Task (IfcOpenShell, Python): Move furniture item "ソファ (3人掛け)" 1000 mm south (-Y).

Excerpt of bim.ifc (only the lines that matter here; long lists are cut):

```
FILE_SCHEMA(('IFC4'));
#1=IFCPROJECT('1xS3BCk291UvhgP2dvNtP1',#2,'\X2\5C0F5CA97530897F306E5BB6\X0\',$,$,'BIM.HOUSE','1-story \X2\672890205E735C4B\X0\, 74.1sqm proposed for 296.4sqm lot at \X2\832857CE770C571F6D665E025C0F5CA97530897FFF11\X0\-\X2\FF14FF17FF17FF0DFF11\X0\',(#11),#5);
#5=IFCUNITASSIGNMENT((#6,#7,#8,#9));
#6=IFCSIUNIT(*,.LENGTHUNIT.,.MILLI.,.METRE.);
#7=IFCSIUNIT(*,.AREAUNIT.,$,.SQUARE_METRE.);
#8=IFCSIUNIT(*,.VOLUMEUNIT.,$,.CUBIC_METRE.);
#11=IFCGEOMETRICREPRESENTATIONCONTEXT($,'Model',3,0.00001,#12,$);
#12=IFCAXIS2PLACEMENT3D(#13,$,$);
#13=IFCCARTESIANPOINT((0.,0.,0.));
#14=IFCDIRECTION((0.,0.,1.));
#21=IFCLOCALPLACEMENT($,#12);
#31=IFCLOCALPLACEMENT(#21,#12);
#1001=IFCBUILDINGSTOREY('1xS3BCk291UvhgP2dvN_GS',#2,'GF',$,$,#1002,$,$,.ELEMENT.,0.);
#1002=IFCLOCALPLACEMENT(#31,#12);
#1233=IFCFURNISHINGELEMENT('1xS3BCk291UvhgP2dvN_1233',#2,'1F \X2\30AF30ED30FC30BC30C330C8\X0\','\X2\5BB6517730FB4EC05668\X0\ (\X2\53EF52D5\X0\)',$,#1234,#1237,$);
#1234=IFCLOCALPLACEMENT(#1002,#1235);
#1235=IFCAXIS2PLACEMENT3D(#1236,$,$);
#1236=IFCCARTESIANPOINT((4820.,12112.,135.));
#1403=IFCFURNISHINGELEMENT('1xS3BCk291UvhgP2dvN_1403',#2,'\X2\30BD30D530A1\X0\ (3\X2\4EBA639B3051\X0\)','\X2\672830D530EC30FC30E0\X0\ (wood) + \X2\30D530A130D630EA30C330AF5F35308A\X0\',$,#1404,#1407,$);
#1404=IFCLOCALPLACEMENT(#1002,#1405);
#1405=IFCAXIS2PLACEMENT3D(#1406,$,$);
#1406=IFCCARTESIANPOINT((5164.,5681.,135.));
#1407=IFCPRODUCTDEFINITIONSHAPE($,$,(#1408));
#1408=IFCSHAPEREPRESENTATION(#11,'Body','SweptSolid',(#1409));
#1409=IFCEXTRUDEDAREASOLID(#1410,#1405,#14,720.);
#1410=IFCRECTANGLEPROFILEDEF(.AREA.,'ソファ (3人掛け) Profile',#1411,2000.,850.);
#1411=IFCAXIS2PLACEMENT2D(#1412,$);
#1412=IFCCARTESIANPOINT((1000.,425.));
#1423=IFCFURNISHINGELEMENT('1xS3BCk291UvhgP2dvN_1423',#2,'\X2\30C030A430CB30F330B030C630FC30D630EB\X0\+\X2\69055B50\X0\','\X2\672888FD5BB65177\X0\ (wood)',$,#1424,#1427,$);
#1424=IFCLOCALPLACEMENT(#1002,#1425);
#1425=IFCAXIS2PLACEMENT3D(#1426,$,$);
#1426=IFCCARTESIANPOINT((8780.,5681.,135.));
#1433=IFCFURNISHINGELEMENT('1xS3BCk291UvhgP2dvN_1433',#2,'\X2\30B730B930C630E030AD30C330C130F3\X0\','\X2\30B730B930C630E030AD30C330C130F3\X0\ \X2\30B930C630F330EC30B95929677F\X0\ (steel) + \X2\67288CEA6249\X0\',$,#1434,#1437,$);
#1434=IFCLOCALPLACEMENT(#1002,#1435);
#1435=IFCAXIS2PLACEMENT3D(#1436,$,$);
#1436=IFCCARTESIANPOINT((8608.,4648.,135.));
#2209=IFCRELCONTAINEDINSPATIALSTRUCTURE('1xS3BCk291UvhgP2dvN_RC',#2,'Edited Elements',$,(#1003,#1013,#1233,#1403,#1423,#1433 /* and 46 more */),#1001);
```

```python
import ifcopenshell
import ifcopenshell.api.geometry
import ifcopenshell.util.placement
import ifcopenshell.util.unit

model = ifcopenshell.open("bim.ifc")
unit_scale = ifcopenshell.util.unit.calculate_unit_scale(model)

item = model.by_id(1403)
matrix = ifcopenshell.util.placement.get_local_placement(item.ObjectPlacement)
matrix[1, 3] -= 1 / unit_scale
ifcopenshell.api.geometry.edit_object_placement(model, product=item, matrix=matrix, is_si=False)

print(ifcopenshell.util.placement.get_local_placement(item.ObjectPlacement).round(3) + 0.0)

model.write("bim_updated.ifc")
```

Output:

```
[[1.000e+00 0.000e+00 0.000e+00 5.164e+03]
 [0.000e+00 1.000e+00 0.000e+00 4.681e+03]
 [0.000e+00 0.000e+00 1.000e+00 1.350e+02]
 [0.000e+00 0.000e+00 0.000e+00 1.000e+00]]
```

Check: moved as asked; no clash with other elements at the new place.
